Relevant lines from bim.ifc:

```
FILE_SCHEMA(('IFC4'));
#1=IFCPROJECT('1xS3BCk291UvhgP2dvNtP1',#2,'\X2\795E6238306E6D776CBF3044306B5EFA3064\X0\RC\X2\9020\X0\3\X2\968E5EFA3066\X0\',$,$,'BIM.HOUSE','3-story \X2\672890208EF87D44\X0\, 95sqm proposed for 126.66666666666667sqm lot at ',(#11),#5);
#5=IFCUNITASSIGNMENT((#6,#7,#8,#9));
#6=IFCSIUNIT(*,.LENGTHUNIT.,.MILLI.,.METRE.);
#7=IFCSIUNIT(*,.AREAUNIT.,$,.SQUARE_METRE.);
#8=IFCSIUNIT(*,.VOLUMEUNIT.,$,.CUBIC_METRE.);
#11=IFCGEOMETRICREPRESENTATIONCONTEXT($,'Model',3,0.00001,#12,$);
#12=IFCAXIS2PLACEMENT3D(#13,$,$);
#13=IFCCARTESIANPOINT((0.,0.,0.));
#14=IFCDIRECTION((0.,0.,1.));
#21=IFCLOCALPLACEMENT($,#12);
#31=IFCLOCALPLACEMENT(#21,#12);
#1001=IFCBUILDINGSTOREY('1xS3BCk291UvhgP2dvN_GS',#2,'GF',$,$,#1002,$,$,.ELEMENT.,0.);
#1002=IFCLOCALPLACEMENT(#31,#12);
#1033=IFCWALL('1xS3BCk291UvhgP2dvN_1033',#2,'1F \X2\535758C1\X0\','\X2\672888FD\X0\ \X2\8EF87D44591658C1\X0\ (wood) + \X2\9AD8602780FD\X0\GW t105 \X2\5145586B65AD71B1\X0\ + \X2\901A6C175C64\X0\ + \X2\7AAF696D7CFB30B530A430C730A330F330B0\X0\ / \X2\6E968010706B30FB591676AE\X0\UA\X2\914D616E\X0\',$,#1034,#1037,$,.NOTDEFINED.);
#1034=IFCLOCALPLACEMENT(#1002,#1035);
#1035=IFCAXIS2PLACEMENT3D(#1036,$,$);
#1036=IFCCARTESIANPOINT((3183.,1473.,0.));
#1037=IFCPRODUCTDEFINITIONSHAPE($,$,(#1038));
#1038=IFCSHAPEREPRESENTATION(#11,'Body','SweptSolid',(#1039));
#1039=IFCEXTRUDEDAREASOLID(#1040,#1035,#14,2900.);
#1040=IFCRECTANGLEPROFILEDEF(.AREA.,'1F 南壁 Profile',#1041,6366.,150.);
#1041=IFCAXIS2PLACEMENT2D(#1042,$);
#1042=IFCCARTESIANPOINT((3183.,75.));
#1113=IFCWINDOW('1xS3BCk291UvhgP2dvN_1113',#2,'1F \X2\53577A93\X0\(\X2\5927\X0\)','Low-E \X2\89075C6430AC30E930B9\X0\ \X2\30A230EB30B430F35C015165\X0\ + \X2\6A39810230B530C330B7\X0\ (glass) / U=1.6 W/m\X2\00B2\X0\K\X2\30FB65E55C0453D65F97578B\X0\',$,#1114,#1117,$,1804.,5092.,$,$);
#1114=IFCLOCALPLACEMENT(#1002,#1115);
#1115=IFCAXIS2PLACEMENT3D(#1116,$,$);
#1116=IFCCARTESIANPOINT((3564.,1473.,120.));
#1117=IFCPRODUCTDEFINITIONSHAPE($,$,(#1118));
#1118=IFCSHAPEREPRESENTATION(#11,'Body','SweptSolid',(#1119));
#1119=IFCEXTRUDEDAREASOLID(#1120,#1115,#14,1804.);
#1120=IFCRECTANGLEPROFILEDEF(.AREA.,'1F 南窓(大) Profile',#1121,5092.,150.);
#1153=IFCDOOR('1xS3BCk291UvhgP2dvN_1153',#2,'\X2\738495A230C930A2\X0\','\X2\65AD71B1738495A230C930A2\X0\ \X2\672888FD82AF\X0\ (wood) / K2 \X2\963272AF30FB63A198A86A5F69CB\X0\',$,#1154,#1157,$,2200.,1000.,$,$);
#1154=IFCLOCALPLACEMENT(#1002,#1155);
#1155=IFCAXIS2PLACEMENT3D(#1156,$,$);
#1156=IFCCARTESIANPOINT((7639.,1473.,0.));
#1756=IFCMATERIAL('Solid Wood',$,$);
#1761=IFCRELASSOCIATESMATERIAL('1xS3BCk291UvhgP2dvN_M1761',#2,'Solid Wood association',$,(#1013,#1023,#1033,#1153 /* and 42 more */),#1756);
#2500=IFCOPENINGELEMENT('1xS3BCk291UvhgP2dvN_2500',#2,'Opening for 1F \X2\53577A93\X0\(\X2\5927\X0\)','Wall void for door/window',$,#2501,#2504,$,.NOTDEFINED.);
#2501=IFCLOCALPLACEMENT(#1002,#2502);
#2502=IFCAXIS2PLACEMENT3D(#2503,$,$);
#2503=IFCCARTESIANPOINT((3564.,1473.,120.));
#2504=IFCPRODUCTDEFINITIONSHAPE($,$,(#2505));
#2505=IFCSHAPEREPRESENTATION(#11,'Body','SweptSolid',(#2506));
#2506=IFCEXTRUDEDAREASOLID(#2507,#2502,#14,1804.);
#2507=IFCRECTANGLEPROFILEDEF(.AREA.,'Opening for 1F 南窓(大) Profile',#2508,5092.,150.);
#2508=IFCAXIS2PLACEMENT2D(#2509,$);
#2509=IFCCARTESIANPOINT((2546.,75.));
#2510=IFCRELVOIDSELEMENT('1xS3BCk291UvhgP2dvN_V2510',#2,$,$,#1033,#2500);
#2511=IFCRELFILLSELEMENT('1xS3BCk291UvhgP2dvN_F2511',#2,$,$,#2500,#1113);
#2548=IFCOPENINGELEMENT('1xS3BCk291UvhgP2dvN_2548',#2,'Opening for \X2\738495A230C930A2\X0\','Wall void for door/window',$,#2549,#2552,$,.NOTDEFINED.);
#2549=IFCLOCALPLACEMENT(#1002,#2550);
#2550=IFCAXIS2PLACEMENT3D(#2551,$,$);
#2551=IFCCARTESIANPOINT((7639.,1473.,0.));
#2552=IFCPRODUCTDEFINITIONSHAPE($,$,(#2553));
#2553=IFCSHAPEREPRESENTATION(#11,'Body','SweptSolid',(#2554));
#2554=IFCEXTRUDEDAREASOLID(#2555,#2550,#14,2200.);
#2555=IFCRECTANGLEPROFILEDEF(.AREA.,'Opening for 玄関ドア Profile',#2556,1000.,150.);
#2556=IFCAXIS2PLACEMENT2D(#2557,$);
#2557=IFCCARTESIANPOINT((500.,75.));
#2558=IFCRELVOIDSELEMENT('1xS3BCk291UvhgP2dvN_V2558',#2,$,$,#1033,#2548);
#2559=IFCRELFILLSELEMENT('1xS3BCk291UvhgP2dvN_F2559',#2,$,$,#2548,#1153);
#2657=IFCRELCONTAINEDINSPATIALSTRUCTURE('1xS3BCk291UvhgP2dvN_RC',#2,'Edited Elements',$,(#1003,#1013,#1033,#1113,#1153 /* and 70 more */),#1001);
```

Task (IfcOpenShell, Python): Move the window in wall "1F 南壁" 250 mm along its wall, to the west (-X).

```python
import ifcopenshell
import ifcopenshell.api.geometry
import ifcopenshell.util.placement
import ifcopenshell.util.unit

model = ifcopenshell.open("bim.ifc")
unit_scale = ifcopenshell.util.unit.calculate_unit_scale(model)

window = model.by_id(1113)
opening = window.FillsVoids[0].RelatingOpeningElement
wall = opening.VoidsElements[0].RelatingBuildingElement

wall_matrix = ifcopenshell.util.placement.get_local_placement(wall.ObjectPlacement)
shift = wall_matrix[:3, 0] * -0.25 / unit_scale
before = ifcopenshell.util.placement.get_local_placement(window.ObjectPlacement)[:3, 3].copy()

# The window is not placed relative to its opening, so move both.
for product in (opening, window):
    matrix = ifcopenshell.util.placement.get_local_placement(product.ObjectPlacement)
    matrix[:3, 3] += shift
    ifcopenshell.api.geometry.edit_object_placement(model, product=product, matrix=matrix, is_si=False)

after = ifcopenshell.util.placement.get_local_placement(window.ObjectPlacement)[:3, 3]
print("window moved by", (after - before).round(3) + 0.0)

model.write("bim-out.ifc")
```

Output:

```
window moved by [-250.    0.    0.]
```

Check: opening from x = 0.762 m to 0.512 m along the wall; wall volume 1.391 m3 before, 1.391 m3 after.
